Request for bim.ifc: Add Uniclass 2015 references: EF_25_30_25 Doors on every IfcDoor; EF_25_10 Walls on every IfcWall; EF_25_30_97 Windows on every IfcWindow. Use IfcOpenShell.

First a look at what the model holds.

```python
import ifcopenshell

model = ifcopenshell.open("bim.ifc")
print(model.schema)
print("classifications:", [c.Name for c in model.by_type("IfcClassification")])
for ifc_class in ("IfcDoor", "IfcRoof", "IfcStair", "IfcWall", "IfcWindow"):
    print(ifc_class, len(model.by_type(ifc_class)))
```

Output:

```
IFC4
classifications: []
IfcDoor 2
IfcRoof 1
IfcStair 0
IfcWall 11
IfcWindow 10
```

```python
import ifcopenshell
import ifcopenshell.api.classification

model = ifcopenshell.open("bim.ifc")

system = ifcopenshell.api.classification.add_classification(model, classification="Uniclass 2015")

codes = {
    "IfcDoor": ("EF_25_30_25", "Doors"),
    "IfcWall": ("EF_25_10", "Walls"),
    "IfcWindow": ("EF_25_30_97", "Windows"),
}
for ifc_class, (code, name) in codes.items():
    products = model.by_type(ifc_class)
    ifcopenshell.api.classification.add_reference(
        model, products=products, classification=system, identification=code, name=name
    )
    print(code, len(products))

model.write("bim_edited.ifc")
```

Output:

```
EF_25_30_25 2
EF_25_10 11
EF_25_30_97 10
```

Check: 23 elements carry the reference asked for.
